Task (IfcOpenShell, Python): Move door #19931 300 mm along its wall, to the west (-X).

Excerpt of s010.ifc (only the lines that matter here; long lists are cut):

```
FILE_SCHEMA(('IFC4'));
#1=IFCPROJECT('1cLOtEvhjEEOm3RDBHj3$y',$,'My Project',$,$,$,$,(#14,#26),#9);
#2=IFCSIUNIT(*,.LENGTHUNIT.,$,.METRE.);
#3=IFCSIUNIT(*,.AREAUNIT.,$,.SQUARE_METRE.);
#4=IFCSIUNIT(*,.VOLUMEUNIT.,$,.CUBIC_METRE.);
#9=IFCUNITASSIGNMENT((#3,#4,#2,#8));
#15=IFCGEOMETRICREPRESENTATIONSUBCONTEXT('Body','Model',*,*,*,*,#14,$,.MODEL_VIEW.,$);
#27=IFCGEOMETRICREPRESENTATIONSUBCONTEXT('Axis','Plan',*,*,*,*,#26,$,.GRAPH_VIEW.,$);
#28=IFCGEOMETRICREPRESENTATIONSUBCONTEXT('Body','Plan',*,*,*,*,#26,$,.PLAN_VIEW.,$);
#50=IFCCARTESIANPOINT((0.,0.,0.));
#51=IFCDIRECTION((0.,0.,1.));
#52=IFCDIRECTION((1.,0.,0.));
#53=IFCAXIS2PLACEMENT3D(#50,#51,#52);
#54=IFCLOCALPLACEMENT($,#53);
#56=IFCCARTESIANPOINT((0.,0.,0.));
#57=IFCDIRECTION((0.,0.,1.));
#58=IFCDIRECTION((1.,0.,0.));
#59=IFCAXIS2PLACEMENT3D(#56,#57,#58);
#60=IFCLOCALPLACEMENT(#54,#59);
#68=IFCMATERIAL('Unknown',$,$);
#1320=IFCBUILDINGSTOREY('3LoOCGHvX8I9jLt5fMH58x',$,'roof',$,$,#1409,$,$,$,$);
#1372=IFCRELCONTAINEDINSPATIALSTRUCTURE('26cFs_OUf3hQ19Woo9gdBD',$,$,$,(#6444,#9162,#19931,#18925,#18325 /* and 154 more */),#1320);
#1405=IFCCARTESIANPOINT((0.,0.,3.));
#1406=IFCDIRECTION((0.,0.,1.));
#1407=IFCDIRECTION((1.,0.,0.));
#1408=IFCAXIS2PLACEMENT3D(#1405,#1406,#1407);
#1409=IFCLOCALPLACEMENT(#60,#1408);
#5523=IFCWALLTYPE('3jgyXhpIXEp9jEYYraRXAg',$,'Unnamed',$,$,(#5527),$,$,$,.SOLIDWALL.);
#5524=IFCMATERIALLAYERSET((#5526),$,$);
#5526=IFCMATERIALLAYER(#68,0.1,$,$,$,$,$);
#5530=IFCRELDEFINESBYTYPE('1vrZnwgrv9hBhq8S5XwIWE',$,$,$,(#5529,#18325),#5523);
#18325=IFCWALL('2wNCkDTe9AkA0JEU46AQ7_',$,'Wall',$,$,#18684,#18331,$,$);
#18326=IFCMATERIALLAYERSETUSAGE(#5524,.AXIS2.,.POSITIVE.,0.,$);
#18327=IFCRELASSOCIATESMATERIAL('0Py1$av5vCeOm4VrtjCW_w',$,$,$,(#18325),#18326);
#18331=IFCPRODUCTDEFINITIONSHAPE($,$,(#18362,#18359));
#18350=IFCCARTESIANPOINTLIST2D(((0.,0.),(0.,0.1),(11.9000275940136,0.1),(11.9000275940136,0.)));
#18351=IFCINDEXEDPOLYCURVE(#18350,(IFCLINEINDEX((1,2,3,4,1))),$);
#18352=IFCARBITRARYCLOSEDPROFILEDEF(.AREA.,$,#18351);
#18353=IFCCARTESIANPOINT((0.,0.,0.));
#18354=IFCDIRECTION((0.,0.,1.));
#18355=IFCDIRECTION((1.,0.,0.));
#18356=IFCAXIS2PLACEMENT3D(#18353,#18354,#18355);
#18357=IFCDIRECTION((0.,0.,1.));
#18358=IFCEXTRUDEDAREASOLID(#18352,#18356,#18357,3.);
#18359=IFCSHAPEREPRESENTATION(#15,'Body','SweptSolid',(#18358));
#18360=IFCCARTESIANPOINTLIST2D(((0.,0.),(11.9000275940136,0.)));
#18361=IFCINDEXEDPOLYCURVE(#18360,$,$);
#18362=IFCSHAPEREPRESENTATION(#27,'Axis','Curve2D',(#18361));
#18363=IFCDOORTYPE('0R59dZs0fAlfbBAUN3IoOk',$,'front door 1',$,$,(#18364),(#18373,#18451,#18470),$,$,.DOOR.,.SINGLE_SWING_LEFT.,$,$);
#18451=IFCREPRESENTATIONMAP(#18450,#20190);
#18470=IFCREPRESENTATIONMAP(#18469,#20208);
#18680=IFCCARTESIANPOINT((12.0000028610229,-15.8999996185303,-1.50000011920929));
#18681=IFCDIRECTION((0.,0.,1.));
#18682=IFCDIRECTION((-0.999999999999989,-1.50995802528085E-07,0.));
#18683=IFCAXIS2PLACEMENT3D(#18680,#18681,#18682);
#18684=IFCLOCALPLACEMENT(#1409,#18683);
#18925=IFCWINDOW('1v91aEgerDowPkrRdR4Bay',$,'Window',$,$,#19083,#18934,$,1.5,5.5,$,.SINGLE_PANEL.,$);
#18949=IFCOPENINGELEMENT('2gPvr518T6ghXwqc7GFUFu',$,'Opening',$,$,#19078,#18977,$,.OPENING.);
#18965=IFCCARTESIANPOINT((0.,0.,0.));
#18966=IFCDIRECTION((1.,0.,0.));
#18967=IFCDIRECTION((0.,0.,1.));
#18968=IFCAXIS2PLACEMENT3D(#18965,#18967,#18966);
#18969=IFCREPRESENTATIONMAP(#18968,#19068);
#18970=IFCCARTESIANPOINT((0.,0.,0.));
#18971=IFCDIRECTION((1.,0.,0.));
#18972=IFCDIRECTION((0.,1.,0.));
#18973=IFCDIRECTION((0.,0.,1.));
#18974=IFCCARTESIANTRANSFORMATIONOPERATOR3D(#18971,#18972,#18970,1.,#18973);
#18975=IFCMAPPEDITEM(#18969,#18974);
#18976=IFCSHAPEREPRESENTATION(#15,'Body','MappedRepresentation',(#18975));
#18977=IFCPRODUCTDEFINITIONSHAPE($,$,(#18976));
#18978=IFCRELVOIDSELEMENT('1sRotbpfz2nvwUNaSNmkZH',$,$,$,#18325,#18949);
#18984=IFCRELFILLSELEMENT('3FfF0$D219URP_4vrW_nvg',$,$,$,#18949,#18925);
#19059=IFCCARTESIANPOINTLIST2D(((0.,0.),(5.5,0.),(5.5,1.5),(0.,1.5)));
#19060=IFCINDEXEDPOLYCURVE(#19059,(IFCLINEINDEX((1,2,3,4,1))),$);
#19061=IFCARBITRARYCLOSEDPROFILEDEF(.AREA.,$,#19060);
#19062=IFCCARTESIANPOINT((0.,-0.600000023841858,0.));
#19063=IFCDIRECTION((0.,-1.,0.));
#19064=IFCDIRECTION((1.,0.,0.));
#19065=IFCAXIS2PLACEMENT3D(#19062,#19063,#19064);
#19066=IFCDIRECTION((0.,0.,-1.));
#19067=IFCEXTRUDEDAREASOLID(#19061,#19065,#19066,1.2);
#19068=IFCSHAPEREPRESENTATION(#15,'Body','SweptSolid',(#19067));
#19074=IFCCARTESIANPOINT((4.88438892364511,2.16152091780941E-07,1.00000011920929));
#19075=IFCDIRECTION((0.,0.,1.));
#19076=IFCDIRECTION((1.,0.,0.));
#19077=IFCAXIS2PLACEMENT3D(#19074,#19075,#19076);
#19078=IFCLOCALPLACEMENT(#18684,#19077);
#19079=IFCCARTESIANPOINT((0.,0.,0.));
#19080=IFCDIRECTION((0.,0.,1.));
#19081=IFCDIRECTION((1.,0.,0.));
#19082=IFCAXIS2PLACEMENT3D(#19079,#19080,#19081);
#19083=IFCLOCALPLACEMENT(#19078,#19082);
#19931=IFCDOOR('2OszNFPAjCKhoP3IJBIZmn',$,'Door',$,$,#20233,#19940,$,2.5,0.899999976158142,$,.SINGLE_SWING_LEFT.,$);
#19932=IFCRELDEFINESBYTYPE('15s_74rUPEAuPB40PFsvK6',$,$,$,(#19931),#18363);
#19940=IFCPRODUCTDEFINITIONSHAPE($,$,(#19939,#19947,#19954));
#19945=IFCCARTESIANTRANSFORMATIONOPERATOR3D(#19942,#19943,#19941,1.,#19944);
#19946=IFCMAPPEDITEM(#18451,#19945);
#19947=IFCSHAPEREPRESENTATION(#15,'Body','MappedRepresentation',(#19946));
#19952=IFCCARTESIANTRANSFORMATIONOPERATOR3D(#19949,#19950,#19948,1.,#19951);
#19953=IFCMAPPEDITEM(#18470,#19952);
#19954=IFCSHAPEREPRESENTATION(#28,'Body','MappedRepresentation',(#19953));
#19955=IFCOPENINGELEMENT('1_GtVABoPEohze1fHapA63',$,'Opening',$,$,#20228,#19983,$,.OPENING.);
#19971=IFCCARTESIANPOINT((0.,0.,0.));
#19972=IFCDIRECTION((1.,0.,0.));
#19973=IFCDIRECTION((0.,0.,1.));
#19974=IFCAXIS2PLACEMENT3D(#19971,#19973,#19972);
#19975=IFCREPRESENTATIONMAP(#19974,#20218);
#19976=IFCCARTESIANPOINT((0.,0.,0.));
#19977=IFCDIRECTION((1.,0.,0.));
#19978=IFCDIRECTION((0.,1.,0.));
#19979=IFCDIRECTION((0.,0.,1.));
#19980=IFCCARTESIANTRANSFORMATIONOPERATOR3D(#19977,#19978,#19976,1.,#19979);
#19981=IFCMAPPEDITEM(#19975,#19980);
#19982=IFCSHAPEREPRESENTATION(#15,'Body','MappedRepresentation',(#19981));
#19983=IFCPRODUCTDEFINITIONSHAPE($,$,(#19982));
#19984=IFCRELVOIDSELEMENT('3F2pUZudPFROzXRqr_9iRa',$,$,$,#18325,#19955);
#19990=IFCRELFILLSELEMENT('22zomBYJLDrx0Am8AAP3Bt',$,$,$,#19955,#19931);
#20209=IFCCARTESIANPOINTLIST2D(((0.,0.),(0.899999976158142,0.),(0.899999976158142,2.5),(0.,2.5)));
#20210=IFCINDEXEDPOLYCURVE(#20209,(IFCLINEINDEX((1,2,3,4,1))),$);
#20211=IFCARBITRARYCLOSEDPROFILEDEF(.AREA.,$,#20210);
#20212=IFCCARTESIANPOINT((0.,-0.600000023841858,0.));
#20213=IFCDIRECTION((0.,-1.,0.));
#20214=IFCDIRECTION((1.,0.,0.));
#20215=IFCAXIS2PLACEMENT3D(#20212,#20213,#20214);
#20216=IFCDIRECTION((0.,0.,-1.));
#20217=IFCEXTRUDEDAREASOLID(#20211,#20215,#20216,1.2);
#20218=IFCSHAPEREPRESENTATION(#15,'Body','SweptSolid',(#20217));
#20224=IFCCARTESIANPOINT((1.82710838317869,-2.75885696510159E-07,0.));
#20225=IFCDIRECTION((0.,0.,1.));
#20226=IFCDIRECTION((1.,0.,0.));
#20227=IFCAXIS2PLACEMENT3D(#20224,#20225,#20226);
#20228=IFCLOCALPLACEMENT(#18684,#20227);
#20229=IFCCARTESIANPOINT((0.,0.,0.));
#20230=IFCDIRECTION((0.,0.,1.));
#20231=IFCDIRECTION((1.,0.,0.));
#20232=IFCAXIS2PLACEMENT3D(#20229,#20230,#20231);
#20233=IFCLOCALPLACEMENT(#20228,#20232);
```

```python
import ifcopenshell
import ifcopenshell.api.geometry
import ifcopenshell.util.placement
import ifcopenshell.util.unit

model = ifcopenshell.open("s010.ifc")
unit_scale = ifcopenshell.util.unit.calculate_unit_scale(model)

door = model.by_guid("2OszNFPAjCKhoP3IJBIZmn")
opening = door.FillsVoids[0].RelatingOpeningElement
wall = opening.VoidsElements[0].RelatingBuildingElement

wall_matrix = ifcopenshell.util.placement.get_local_placement(wall.ObjectPlacement)
shift = wall_matrix[:3, 0] * 0.3 / unit_scale
before = ifcopenshell.util.placement.get_local_placement(door.ObjectPlacement)[:3, 3].copy()

# The door is placed relative to its opening, so it follows when the opening moves.
matrix = ifcopenshell.util.placement.get_local_placement(opening.ObjectPlacement)
matrix[:3, 3] += shift
ifcopenshell.api.geometry.edit_object_placement(
    model, product=opening, matrix=matrix, is_si=False, should_transform_children=True
)

after = ifcopenshell.util.placement.get_local_placement(door.ObjectPlacement)[:3, 3]
print("door moved by", (after - before).round(3) + 0.0)

model.write("s010_updated.ifc")
```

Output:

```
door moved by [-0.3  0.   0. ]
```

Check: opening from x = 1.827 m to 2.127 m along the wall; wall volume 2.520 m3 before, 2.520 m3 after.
